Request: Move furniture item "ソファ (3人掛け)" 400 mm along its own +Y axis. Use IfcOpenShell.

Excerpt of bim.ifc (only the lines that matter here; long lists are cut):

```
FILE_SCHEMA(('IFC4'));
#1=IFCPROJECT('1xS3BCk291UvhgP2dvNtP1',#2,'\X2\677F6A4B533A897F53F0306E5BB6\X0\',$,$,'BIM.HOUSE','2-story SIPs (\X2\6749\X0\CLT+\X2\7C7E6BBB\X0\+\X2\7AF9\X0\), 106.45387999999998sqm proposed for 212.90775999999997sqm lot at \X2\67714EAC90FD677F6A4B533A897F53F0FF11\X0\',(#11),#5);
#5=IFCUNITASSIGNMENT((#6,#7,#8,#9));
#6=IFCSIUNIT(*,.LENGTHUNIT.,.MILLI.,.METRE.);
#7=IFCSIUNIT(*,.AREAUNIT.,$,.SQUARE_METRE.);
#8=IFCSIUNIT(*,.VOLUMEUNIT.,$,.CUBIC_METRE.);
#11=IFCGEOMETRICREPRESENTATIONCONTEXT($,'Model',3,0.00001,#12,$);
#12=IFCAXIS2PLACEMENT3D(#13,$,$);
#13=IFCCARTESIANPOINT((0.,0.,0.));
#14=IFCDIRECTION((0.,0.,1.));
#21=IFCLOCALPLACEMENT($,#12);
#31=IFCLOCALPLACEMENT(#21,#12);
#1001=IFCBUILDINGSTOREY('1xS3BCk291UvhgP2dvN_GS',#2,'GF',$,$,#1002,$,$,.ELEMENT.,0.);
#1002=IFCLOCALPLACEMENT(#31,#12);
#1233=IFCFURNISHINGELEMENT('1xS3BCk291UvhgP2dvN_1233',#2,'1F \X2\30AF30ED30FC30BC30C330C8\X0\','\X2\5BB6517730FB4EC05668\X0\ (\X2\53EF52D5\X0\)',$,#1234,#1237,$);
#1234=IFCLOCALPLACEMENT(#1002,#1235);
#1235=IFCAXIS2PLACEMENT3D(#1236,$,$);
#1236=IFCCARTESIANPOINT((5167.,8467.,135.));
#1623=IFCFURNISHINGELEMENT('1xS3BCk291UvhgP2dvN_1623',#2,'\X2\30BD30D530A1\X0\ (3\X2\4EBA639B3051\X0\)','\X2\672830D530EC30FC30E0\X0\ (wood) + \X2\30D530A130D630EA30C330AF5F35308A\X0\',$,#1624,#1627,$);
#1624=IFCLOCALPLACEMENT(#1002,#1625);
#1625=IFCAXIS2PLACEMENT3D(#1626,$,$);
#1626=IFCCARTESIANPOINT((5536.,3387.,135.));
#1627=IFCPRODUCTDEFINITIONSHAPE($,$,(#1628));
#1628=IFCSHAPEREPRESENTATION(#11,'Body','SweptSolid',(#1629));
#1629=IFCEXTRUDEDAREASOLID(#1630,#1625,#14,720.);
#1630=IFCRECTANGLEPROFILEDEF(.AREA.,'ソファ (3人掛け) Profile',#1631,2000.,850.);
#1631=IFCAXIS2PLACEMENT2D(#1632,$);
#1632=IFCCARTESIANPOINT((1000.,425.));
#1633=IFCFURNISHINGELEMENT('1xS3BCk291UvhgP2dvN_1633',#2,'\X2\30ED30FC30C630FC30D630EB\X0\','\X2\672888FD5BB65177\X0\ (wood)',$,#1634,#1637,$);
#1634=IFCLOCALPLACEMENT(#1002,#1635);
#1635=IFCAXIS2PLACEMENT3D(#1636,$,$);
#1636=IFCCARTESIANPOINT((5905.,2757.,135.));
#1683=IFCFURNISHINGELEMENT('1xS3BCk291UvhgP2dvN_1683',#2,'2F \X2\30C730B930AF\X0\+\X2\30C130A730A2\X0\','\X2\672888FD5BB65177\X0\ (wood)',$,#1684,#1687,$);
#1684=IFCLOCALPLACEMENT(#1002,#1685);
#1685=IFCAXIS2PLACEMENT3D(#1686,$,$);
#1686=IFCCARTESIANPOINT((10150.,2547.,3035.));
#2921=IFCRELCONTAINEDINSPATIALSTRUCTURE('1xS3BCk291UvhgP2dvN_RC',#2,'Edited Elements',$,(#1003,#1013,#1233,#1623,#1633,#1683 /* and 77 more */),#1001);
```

```python
import ifcopenshell
import ifcopenshell.api.geometry
import ifcopenshell.util.placement
import ifcopenshell.util.unit

model = ifcopenshell.open("bim.ifc")
unit_scale = ifcopenshell.util.unit.calculate_unit_scale(model)

item = model.by_guid("1xS3BCk291UvhgP2dvN_1623")
matrix = ifcopenshell.util.placement.get_local_placement(item.ObjectPlacement)
matrix[:3, 3] += matrix[:3, 1] * 0.4 / unit_scale
ifcopenshell.api.geometry.edit_object_placement(model, product=item, matrix=matrix, is_si=False)

print(ifcopenshell.util.placement.get_local_placement(item.ObjectPlacement).round(3) + 0.0)

model.write("bim_rev.ifc")
```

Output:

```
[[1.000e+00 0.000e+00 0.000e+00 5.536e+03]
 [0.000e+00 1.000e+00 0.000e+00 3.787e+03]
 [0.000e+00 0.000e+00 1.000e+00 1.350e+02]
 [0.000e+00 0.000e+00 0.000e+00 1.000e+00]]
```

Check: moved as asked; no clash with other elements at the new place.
